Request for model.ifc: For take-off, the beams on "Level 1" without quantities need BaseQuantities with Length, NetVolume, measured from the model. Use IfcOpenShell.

First a look at what the model holds.

```python
import ifcopenshell
import ifcopenshell.util.element
import ifcopenshell.util.unit

model = ifcopenshell.open("model.ifc")
print(model.schema)
for unit_type in ("LENGTHUNIT", "AREAUNIT", "VOLUMEUNIT"):
    print(unit_type, ifcopenshell.util.unit.calculate_unit_scale(model, unit_type))
storey = next(s for s in model.by_type("IfcBuildingStorey") if s.Name == "Level 1")
beams = [e for e in ifcopenshell.util.element.get_decomposition(storey) if e.is_a("IfcBeam")]
for e in sorted(beams, key=lambda e: e.id()):
    print(e.id(), e.is_a(), e.Name, list(ifcopenshell.util.element.get_psets(e, qtos_only=True)), sep=" | ")
```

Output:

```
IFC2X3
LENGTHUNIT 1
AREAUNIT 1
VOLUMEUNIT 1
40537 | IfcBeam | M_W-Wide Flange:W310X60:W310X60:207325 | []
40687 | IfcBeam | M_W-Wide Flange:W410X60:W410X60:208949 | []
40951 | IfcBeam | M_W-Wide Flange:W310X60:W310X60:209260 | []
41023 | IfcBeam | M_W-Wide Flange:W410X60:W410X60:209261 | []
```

```python
import ifcopenshell
import ifcopenshell.api.pset
import ifcopenshell.geom
import ifcopenshell.util.element
import ifcopenshell.util.shape
import ifcopenshell.util.unit

model = ifcopenshell.open("model.ifc")
unit_scale = ifcopenshell.util.unit.calculate_unit_scale(model)
volume_scale = ifcopenshell.util.unit.calculate_unit_scale(model, "VOLUMEUNIT")
settings = ifcopenshell.geom.settings()

storey = next(s for s in model.by_type("IfcBuildingStorey") if s.Name == "Level 1")
beams = [e for e in ifcopenshell.util.element.get_decomposition(storey) if e.is_a("IfcBeam")]

for e in sorted(beams, key=lambda e: e.id()):
    if ifcopenshell.util.element.get_psets(e, qtos_only=True, should_inherit=False):
        continue
    # Geometry comes back in metres, in the element's own axes.
    shape = ifcopenshell.geom.create_shape(settings, e)
    values = {
        "Length": ifcopenshell.util.shape.get_max_xyz(shape.geometry) / unit_scale,
        "NetVolume": ifcopenshell.util.shape.get_volume(shape.geometry) / volume_scale,
    }
    qto = ifcopenshell.api.pset.add_qto(model, product=e, name="BaseQuantities")
    ifcopenshell.api.pset.edit_qto(model, qto=qto, properties=values)
    print(e.id(), {k: round(v, 3) for k, v in values.items()})

model.write("model_edited.ifc")
```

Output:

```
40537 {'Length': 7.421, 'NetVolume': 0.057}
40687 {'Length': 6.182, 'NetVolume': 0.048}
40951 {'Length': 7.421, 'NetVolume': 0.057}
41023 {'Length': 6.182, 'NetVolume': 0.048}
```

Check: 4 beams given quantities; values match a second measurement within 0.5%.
